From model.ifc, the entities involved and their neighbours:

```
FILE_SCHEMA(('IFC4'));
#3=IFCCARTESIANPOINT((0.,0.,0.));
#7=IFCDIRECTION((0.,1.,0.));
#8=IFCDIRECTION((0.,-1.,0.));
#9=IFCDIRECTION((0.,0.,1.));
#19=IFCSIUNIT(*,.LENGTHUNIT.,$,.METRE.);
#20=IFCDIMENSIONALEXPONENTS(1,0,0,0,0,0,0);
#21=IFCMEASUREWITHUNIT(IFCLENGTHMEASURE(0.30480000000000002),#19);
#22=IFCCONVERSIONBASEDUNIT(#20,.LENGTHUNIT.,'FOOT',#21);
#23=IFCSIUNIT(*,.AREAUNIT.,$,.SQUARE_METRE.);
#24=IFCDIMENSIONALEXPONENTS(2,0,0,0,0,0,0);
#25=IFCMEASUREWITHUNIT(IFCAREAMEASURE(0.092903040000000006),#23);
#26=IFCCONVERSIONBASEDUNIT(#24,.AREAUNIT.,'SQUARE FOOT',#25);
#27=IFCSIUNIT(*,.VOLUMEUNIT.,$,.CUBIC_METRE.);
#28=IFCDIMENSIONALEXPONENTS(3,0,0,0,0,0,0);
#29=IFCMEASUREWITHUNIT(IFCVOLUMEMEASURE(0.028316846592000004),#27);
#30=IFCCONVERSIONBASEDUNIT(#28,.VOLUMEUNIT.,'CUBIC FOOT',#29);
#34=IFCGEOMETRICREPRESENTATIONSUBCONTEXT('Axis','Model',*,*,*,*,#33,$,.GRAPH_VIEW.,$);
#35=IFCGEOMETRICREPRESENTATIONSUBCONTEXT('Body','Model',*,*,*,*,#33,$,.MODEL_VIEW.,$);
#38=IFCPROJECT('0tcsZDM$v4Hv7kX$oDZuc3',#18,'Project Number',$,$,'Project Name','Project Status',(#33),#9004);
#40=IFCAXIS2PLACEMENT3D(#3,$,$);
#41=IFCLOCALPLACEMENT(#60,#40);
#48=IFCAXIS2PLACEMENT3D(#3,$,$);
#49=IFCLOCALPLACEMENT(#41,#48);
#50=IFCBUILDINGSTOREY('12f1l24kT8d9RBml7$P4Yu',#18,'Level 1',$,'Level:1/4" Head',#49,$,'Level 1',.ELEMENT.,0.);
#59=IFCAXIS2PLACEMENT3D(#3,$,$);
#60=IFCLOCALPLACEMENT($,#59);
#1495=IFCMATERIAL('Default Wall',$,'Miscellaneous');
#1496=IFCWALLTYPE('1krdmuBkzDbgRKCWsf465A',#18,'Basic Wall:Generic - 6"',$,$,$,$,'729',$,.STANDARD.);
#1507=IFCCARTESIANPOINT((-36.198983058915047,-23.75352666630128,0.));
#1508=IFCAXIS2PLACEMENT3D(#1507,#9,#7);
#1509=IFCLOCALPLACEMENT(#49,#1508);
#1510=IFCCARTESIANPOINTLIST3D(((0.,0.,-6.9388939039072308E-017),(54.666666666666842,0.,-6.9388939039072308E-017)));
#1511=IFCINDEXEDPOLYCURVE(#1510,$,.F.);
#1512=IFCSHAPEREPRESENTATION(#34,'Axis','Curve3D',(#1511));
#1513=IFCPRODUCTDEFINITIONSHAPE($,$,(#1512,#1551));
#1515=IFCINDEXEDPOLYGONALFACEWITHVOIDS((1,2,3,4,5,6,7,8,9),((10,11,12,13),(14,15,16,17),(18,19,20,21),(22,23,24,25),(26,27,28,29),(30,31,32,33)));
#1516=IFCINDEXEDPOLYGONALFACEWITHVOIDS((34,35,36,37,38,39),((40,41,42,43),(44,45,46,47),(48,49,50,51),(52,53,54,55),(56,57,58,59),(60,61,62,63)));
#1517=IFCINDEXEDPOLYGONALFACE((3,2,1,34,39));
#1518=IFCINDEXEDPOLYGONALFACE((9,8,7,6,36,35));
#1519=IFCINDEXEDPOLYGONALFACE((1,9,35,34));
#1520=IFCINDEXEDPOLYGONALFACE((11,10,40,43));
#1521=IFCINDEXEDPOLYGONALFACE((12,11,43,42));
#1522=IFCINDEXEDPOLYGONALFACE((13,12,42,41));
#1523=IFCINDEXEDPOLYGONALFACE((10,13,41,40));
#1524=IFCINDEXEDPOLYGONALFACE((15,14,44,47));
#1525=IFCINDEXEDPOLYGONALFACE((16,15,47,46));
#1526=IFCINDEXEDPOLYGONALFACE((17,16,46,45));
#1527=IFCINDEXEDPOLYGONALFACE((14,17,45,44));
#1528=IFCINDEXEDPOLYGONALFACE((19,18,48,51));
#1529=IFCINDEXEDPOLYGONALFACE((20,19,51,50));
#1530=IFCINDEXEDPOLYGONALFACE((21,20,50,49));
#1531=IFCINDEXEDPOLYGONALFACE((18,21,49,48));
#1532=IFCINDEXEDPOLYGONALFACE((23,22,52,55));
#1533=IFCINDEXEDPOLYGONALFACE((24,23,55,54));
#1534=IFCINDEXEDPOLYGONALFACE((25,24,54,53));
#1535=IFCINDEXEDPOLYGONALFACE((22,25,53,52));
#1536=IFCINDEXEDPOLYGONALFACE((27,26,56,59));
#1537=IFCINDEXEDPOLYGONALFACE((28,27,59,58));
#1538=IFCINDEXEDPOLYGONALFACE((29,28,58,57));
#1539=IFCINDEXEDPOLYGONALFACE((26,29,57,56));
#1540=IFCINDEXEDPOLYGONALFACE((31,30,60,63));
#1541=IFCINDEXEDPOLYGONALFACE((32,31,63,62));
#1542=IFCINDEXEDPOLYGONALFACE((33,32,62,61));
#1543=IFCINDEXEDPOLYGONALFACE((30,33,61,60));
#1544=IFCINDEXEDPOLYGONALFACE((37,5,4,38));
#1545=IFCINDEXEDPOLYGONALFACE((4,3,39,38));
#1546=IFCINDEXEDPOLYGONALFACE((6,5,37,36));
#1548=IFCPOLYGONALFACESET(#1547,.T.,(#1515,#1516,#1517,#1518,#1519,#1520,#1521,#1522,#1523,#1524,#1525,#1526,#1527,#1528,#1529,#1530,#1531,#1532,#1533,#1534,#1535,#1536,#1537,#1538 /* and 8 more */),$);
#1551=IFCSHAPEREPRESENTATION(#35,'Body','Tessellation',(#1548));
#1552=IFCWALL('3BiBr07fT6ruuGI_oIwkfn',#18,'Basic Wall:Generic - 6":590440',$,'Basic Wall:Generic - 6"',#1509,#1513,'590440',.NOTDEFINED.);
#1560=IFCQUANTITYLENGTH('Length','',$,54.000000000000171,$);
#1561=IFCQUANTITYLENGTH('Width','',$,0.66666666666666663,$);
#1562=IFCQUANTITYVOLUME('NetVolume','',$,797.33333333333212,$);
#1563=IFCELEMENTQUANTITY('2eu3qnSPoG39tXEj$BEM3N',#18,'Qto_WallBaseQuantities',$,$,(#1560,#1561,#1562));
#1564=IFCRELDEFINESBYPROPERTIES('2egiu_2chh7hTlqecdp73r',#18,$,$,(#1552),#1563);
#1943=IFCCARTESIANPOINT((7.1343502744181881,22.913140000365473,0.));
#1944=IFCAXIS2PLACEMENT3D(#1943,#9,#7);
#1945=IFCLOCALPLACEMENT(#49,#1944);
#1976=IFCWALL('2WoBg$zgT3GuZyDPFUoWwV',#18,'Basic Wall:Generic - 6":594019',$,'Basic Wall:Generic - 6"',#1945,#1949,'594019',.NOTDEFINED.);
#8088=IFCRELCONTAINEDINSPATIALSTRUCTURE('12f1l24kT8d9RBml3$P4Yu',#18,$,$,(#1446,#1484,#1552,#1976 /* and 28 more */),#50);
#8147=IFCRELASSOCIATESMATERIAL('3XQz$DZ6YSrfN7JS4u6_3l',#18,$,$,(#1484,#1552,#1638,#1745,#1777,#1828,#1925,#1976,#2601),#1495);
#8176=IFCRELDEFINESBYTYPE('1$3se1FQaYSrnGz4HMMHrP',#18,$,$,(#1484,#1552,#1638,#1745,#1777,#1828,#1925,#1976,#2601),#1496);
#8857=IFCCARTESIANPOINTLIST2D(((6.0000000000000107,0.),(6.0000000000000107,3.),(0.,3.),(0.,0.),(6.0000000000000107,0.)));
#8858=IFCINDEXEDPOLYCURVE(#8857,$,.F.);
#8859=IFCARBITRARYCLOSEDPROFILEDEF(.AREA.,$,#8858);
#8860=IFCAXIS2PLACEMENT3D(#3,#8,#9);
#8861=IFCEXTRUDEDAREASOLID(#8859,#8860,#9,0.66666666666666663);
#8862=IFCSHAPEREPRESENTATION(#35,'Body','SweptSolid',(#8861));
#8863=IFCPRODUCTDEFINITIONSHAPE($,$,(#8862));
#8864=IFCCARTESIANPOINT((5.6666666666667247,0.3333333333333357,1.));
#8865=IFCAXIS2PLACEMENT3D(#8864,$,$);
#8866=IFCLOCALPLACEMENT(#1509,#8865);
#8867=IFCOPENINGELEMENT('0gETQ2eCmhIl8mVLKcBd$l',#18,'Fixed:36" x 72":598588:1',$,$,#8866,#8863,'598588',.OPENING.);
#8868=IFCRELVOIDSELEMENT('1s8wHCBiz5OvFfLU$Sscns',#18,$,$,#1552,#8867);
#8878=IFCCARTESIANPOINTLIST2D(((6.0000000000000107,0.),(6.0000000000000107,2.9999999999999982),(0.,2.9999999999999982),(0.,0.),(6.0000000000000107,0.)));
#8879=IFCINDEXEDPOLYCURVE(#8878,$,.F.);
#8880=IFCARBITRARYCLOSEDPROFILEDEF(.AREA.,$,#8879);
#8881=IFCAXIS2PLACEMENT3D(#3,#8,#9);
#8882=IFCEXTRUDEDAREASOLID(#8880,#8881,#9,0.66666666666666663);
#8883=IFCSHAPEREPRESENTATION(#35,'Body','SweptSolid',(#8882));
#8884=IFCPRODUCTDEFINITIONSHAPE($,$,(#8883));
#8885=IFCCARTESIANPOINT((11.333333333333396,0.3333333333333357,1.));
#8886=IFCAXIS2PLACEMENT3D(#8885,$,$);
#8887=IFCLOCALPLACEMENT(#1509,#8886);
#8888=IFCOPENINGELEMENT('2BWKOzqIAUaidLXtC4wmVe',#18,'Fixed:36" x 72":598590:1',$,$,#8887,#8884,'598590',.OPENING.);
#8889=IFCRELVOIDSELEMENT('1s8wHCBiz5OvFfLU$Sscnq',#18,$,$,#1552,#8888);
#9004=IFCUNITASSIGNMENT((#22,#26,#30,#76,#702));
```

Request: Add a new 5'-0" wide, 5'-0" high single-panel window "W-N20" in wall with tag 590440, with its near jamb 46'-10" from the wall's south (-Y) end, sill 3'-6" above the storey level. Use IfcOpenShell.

```python
import numpy as np
import ifcopenshell
import ifcopenshell.api.feature
import ifcopenshell.api.geometry
import ifcopenshell.api.pset
import ifcopenshell.api.root
import ifcopenshell.api.spatial
import ifcopenshell.geom
import ifcopenshell.util.element
import ifcopenshell.util.placement
import ifcopenshell.util.representation
import ifcopenshell.util.shape
import ifcopenshell.util.unit

model = ifcopenshell.open("model.ifc")
unit_scale = ifcopenshell.util.unit.calculate_unit_scale(model)
volume_scale = ifcopenshell.util.unit.calculate_unit_scale(model, "VOLUMEUNIT")
settings = ifcopenshell.geom.settings()


def volume(element):
    """Net volume in cubic metres, openings subtracted."""
    shape = ifcopenshell.geom.create_shape(settings, element)
    return ifcopenshell.util.shape.get_volume(shape.geometry)


wall = model.by_guid("3BiBr07fT6ruuGI_oIwkfn")
storey = ifcopenshell.util.element.get_container(wall, ifc_class="IfcBuildingStorey")
context = ifcopenshell.util.representation.get_context(model, "Model", "Body", "MODEL_VIEW")
before = volume(wall)

width, height, from_end, sill = 1.524, 1.524, 14.2748, 1.0668  # metres

# The wall runs along its own X axis, and the end named is its -X end.
wall_shape = ifcopenshell.geom.create_shape(settings, wall)
x, y, z = ifcopenshell.util.shape.get_vertices(wall_shape.geometry).T
start = x.min() + from_end
face, thickness = float(y.min()), float(y.max() - y.min())
wall_matrix = ifcopenshell.util.placement.get_local_placement(wall.ObjectPlacement)
level = ifcopenshell.util.placement.get_local_placement(storey.ObjectPlacement)[2, 3]


def in_wall(x, y):
    """Placement at x, y metres in the wall's axes, at sill height."""
    matrix = wall_matrix.copy()
    matrix[:, 3] = wall_matrix @ np.array([x / unit_scale, y / unit_scale, 0.0, 1.0])
    matrix[2, 3] = level + sill / unit_scale
    return matrix


# Opening: a box that overshoots both wall faces by 50 mm.
opening = ifcopenshell.api.root.create_entity(model, ifc_class="IfcOpeningElement", predefined_type="OPENING")
box = ifcopenshell.api.geometry.add_wall_representation(
    model, context=context, length=width, height=height, thickness=thickness + 0.1
)
ifcopenshell.api.geometry.assign_representation(model, product=opening, representation=box)
ifcopenshell.api.geometry.edit_object_placement(model, product=opening, matrix=in_wall(start, face - 0.05), is_si=False)
ifcopenshell.api.feature.add_feature(model, feature=opening, element=wall)

window = ifcopenshell.api.root.create_entity(model, ifc_class="IfcWindow", name="W-N20", predefined_type="WINDOW")
window.OverallWidth, window.OverallHeight = width / unit_scale, height / unit_scale
window.PartitioningType = "SINGLE_PANEL"
body = ifcopenshell.api.geometry.add_window_representation(
    model,
    context=context,
    overall_width=window.OverallWidth,
    overall_height=window.OverallHeight,
    partition_type="SINGLE_PANEL",
)
ifcopenshell.api.geometry.assign_representation(model, product=window, representation=body)
ifcopenshell.api.spatial.assign_container(model, products=[window], relating_structure=storey)
ifcopenshell.api.feature.add_filling(model, opening=opening, element=window)

# Centre the window in the wall's thickness.
ifcopenshell.api.geometry.edit_object_placement(model, product=window, matrix=in_wall(start, face), is_si=False)
window_shape = ifcopenshell.geom.create_shape(settings, window)
depth = ifcopenshell.util.shape.get_vertices(window_shape.geometry)[:, 1]
offset = face + thickness / 2 - (depth.min() + depth.max()) / 2
ifcopenshell.api.geometry.edit_object_placement(model, product=window, matrix=in_wall(start, offset), is_si=False)

after = volume(wall)

# Update the wall's stored quantities.
qto = model.by_id(ifcopenshell.util.element.get_pset(wall, "Qto_WallBaseQuantities", should_inherit=False)["id"])
ifcopenshell.api.pset.edit_qto(model, qto=qto, properties={"NetVolume": after / volume_scale})

print(f"wall volume {before:.3f} -> {after:.3f} m3")

model.write("model-out.ifc")
```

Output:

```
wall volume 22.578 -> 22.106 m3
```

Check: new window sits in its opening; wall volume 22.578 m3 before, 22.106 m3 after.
